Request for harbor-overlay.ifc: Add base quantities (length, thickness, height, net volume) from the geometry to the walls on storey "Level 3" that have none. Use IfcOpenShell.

First a look at what the model holds.

```python
import ifcopenshell
import ifcopenshell.util.element
import ifcopenshell.util.unit

model = ifcopenshell.open("harbor-overlay.ifc")
print(model.schema)
for unit_type in ("LENGTHUNIT", "AREAUNIT", "VOLUMEUNIT"):
    print(unit_type, ifcopenshell.util.unit.calculate_unit_scale(model, unit_type))
storey = next(s for s in model.by_type("IfcBuildingStorey") if s.Name == "Level 3")
walls = [e for e in ifcopenshell.util.element.get_decomposition(storey) if e.is_a("IfcWall")]
for e in sorted(walls, key=lambda e: e.id()):
    print(e.id(), e.is_a(), e.Name, list(ifcopenshell.util.element.get_psets(e, qtos_only=True)), sep=" | ")
```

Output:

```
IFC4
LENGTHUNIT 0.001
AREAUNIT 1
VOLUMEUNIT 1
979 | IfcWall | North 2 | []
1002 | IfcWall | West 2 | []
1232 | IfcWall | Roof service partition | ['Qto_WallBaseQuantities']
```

```python
import ifcopenshell
import ifcopenshell.api.pset
import ifcopenshell.geom
import ifcopenshell.util.element
import ifcopenshell.util.shape
import ifcopenshell.util.unit

model = ifcopenshell.open("harbor-overlay.ifc")
unit_scale = ifcopenshell.util.unit.calculate_unit_scale(model)
volume_scale = ifcopenshell.util.unit.calculate_unit_scale(model, "VOLUMEUNIT")
settings = ifcopenshell.geom.settings()

storey = next(s for s in model.by_type("IfcBuildingStorey") if s.Name == "Level 3")
walls = [e for e in ifcopenshell.util.element.get_decomposition(storey) if e.is_a("IfcWall")]

for e in sorted(walls, key=lambda e: e.id()):
    if ifcopenshell.util.element.get_psets(e, qtos_only=True, should_inherit=False):
        continue
    # Geometry comes back in metres, in the element's own axes.
    shape = ifcopenshell.geom.create_shape(settings, e)
    values = {
        "Length": ifcopenshell.util.shape.get_x(shape.geometry) / unit_scale,
        "Width": ifcopenshell.util.shape.get_y(shape.geometry) / unit_scale,
        "Height": ifcopenshell.util.shape.get_z(shape.geometry) / unit_scale,
        "NetVolume": ifcopenshell.util.shape.get_volume(shape.geometry) / volume_scale,
    }
    qto = ifcopenshell.api.pset.add_qto(model, product=e, name="Qto_WallBaseQuantities")
    ifcopenshell.api.pset.edit_qto(model, qto=qto, properties=values)
    print(e.id(), {k: round(v, 3) for k, v in values.items()})

model.write("harbor-overlay_edited.ifc")
```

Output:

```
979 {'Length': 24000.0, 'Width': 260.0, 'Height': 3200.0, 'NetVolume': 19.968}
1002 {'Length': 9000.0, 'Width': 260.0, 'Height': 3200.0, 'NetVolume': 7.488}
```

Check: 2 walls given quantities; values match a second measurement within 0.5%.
